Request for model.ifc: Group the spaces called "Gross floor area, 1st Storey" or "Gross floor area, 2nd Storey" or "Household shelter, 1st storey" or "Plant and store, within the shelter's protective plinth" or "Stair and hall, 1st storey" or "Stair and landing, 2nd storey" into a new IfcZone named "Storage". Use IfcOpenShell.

First a look at what the model holds.

```python
import ifcopenshell

model = ifcopenshell.open("model.ifc")
print(model.schema)
seen = {}
for space in model.by_type("IfcSpace"):
    seen[space.LongName] = seen.get(space.LongName, 0) + 1
for name, count in sorted(seen.items(), key=str):
    print(count, "x", name)
print("zones:", [z.Name for z in model.by_type("IfcZone")][:20])
```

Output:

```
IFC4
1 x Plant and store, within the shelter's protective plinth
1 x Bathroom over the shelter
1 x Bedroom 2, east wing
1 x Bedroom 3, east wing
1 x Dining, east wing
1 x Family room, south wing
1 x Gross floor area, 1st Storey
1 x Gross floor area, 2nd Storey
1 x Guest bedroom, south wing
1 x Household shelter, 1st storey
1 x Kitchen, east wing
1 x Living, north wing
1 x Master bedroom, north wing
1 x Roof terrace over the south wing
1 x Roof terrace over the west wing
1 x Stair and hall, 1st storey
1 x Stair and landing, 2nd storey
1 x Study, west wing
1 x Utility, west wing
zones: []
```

```python
import ifcopenshell
import ifcopenshell.api.group
import ifcopenshell.api.root

model = ifcopenshell.open("model.ifc")

names = {"Gross floor area, 1st Storey", "Gross floor area, 2nd Storey", "Household shelter, 1st storey", "Plant and store, within the shelter's protective plinth", "Stair and hall, 1st storey", "Stair and landing, 2nd storey"}
spaces = [s for s in model.by_type("IfcSpace") if s.LongName in names]

zone = ifcopenshell.api.root.create_entity(model, ifc_class="IfcZone", name="Storage")
ifcopenshell.api.group.assign_group(model, products=spaces, group=zone)
print(len(spaces), "spaces in", zone.Name)

model.write("model_rev.ifc")
```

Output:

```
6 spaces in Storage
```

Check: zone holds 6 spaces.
